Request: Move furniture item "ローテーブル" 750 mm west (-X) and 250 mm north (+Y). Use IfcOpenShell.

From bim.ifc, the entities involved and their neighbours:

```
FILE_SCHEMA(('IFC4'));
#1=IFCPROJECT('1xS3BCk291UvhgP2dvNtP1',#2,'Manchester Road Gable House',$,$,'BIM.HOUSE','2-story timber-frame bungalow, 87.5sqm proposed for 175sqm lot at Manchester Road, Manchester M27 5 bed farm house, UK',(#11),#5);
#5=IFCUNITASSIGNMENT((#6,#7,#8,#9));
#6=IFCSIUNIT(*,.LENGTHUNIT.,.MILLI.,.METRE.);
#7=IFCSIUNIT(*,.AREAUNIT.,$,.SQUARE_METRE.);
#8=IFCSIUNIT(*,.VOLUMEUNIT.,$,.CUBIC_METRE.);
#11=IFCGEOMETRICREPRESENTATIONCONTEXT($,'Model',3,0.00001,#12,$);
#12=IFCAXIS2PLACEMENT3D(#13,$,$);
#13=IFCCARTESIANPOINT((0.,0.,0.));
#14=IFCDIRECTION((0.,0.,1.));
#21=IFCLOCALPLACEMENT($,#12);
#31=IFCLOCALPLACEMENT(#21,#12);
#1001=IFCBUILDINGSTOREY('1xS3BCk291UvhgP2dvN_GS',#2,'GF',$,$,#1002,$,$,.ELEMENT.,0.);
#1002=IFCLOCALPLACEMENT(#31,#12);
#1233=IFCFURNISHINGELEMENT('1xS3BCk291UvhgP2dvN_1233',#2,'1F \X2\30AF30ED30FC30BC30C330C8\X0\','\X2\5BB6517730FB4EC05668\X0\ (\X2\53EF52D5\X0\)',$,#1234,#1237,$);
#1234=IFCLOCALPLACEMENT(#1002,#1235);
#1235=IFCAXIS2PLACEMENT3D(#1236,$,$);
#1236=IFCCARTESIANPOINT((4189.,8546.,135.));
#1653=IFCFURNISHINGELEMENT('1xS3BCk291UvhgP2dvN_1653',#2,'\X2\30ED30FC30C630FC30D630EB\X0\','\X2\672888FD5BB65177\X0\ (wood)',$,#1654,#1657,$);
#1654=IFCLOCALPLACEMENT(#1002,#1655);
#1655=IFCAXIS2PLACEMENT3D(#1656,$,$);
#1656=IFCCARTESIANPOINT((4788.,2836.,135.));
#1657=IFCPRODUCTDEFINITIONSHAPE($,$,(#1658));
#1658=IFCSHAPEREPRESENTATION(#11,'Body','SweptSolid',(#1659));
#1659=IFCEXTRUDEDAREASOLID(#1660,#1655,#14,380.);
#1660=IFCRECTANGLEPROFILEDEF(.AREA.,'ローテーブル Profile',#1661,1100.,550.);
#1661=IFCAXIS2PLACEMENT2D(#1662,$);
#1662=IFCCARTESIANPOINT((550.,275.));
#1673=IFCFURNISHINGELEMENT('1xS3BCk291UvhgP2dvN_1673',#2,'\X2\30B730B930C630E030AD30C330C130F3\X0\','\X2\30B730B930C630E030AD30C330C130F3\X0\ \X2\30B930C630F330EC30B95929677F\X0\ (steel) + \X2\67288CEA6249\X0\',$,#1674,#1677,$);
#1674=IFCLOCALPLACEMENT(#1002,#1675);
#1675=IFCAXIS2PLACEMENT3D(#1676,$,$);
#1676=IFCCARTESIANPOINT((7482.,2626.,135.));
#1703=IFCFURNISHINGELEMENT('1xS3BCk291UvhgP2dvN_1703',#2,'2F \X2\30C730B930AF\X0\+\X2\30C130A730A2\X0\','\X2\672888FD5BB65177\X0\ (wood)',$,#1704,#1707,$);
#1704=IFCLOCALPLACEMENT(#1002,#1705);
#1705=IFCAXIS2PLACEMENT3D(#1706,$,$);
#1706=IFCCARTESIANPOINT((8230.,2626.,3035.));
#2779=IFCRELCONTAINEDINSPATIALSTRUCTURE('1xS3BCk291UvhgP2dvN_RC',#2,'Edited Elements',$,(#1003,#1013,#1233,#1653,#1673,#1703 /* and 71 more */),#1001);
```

```python
import ifcopenshell
import ifcopenshell.api.geometry
import ifcopenshell.util.placement

model = ifcopenshell.open("bim.ifc")

item = model.by_guid("1xS3BCk291UvhgP2dvN_1653")
matrix = ifcopenshell.util.placement.get_local_placement(item.ObjectPlacement)
matrix[0, 3] -= 750.0
matrix[1, 3] += 250.0
ifcopenshell.api.geometry.edit_object_placement(model, product=item, matrix=matrix, is_si=False)

print(ifcopenshell.util.placement.get_local_placement(item.ObjectPlacement).round(3) + 0.0)

model.write("bim_edited.ifc")
```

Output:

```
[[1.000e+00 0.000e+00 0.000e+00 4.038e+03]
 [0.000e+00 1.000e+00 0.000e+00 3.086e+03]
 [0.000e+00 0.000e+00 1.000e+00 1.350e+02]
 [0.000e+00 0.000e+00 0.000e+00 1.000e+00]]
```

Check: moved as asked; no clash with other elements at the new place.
